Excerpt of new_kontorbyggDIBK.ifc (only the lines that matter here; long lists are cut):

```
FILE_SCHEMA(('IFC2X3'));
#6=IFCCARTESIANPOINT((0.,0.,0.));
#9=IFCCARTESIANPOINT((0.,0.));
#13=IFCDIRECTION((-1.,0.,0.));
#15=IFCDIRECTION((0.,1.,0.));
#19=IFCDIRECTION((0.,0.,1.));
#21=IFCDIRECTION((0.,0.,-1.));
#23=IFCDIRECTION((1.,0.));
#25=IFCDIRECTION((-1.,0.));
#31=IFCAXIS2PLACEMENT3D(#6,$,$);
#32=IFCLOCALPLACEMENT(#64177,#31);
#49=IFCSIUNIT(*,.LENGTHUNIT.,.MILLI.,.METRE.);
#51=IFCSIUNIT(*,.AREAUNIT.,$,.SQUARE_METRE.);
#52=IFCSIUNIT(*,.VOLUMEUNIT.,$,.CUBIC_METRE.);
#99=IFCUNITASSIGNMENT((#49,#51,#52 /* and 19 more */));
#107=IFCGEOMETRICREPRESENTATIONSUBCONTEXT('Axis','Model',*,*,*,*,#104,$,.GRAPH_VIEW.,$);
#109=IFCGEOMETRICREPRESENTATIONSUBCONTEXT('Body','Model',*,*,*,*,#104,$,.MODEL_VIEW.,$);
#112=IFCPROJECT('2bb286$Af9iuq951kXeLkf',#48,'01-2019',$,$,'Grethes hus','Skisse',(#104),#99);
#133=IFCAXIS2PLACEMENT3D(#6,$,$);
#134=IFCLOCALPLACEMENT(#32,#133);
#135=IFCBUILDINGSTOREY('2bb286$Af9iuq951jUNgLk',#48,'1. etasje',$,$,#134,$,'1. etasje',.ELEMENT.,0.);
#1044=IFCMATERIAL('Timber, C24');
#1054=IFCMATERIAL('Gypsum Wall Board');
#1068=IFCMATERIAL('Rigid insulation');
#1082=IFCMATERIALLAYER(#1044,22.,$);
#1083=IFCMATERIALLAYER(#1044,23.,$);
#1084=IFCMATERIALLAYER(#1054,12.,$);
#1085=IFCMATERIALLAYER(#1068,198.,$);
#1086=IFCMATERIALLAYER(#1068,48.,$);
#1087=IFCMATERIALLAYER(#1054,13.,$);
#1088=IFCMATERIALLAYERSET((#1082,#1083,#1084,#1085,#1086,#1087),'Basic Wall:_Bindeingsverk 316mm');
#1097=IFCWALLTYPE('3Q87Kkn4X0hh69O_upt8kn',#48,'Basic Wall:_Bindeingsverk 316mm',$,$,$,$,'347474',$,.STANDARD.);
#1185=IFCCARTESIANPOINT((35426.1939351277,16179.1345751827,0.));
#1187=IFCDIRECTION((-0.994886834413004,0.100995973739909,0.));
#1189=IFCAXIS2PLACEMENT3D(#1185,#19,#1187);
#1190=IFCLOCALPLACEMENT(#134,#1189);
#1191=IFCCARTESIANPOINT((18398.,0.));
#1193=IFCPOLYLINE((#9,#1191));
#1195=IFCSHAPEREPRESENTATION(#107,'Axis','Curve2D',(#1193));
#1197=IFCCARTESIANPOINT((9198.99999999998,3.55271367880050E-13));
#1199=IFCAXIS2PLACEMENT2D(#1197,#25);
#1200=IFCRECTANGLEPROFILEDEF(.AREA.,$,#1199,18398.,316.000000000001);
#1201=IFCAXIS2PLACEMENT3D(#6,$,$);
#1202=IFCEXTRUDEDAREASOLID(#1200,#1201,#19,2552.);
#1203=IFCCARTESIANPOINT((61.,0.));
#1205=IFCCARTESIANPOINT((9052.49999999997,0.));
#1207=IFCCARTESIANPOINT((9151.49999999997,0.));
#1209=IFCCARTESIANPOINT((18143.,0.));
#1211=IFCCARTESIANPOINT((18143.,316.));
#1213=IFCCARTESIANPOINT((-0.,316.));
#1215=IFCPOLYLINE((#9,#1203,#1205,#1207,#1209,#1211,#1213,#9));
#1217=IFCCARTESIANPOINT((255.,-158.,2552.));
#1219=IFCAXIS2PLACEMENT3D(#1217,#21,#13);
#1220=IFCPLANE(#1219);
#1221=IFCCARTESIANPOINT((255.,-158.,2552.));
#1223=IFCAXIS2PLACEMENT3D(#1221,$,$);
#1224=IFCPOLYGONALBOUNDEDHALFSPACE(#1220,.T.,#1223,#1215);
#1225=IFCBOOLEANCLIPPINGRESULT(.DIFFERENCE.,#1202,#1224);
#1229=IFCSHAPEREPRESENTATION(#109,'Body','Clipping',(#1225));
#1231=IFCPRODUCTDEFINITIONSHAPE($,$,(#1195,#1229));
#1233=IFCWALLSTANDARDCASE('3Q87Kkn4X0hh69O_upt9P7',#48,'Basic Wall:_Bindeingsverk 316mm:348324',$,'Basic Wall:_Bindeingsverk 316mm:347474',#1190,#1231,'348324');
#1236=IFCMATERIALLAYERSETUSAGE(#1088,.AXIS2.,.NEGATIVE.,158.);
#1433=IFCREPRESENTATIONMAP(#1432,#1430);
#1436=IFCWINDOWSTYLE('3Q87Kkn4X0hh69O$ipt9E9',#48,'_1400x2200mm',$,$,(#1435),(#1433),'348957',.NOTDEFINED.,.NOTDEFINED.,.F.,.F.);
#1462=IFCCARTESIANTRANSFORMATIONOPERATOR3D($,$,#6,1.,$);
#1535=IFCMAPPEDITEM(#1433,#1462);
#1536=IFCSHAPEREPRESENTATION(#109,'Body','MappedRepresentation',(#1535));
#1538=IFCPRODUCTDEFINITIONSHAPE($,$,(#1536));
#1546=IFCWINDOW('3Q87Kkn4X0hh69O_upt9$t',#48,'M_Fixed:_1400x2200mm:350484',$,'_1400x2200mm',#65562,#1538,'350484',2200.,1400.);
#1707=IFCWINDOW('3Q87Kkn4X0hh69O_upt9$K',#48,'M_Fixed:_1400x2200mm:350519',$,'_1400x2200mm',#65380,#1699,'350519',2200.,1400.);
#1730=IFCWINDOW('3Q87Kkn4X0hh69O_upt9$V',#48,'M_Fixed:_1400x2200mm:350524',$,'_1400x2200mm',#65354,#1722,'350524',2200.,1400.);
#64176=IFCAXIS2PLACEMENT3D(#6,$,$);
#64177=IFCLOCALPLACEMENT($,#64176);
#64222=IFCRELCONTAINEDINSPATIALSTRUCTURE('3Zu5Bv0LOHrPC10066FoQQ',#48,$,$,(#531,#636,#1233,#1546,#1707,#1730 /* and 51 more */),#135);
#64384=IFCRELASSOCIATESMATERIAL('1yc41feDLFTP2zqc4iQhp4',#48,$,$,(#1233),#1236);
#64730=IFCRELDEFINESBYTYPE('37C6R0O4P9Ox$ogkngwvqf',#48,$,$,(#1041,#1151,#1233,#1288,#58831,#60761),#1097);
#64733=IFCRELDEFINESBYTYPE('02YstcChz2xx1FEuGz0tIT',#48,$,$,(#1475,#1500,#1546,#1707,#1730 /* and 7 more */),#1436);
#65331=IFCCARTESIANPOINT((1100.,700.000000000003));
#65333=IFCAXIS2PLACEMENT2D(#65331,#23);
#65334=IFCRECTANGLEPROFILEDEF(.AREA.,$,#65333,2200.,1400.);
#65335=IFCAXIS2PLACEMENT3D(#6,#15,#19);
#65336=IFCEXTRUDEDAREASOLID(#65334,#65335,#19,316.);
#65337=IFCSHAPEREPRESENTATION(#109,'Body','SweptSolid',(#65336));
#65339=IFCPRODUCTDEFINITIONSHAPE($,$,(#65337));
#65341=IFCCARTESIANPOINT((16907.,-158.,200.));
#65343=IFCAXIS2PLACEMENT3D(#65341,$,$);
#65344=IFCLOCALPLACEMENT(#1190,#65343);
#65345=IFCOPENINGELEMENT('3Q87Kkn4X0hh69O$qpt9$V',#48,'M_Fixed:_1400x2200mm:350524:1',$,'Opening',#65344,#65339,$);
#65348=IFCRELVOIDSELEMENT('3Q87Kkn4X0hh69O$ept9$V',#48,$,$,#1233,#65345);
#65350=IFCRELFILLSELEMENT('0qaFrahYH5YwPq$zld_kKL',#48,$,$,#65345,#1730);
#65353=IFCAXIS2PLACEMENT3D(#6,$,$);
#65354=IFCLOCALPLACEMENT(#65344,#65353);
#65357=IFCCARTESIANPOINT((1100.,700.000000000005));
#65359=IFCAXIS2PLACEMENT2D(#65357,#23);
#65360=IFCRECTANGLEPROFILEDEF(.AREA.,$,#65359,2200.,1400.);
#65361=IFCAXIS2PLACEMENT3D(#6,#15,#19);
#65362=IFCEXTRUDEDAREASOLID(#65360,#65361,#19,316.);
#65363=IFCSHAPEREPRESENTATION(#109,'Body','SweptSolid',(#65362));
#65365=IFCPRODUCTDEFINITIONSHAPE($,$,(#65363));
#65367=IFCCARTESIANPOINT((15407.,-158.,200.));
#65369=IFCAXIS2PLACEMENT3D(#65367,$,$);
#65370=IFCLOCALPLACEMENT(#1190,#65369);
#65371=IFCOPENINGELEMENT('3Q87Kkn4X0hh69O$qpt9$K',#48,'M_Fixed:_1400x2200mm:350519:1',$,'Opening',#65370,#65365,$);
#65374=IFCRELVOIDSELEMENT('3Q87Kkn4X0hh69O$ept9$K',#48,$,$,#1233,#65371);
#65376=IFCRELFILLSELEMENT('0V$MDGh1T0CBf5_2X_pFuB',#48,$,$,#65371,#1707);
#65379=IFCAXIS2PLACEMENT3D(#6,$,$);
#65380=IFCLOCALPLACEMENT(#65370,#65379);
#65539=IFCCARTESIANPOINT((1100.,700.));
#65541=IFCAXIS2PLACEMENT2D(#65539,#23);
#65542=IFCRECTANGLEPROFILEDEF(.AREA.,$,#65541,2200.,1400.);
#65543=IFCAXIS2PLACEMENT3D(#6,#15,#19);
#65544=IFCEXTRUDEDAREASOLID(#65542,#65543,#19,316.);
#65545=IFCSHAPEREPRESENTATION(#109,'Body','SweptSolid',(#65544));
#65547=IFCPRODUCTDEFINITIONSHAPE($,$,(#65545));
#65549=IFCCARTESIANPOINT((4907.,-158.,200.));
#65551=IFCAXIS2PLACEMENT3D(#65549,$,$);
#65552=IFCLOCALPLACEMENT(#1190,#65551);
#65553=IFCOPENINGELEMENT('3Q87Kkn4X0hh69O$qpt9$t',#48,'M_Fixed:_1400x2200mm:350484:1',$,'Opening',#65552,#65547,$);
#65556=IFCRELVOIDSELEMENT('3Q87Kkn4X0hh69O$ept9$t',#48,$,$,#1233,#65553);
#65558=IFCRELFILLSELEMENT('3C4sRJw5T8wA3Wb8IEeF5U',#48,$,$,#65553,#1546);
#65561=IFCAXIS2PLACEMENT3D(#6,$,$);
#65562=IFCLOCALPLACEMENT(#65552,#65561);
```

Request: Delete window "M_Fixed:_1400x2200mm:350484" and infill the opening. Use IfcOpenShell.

```python
import ifcopenshell
import ifcopenshell.api.feature
import ifcopenshell.api.root
import ifcopenshell.geom
import ifcopenshell.util.shape

model = ifcopenshell.open("new_kontorbyggDIBK.ifc")
settings = ifcopenshell.geom.settings()


def volume(element):
    """Net volume in cubic metres, openings subtracted."""
    shape = ifcopenshell.geom.create_shape(settings, element)
    return ifcopenshell.util.shape.get_volume(shape.geometry)


window = model.by_guid("3Q87Kkn4X0hh69O_upt9$t")
opening = window.FillsVoids[0].RelatingOpeningElement
wall = opening.VoidsElements[0].RelatingBuildingElement
before = volume(wall)

ifcopenshell.api.root.remove_product(model, product=window)
ifcopenshell.api.feature.remove_feature(model, feature=opening)

after = volume(wall)

print(f"wall volume {before:.3f} -> {after:.3f} m3")

model.write("new_kontorbyggDIBK_v2.ifc")
```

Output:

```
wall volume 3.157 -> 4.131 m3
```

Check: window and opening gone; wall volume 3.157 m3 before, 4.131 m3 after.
